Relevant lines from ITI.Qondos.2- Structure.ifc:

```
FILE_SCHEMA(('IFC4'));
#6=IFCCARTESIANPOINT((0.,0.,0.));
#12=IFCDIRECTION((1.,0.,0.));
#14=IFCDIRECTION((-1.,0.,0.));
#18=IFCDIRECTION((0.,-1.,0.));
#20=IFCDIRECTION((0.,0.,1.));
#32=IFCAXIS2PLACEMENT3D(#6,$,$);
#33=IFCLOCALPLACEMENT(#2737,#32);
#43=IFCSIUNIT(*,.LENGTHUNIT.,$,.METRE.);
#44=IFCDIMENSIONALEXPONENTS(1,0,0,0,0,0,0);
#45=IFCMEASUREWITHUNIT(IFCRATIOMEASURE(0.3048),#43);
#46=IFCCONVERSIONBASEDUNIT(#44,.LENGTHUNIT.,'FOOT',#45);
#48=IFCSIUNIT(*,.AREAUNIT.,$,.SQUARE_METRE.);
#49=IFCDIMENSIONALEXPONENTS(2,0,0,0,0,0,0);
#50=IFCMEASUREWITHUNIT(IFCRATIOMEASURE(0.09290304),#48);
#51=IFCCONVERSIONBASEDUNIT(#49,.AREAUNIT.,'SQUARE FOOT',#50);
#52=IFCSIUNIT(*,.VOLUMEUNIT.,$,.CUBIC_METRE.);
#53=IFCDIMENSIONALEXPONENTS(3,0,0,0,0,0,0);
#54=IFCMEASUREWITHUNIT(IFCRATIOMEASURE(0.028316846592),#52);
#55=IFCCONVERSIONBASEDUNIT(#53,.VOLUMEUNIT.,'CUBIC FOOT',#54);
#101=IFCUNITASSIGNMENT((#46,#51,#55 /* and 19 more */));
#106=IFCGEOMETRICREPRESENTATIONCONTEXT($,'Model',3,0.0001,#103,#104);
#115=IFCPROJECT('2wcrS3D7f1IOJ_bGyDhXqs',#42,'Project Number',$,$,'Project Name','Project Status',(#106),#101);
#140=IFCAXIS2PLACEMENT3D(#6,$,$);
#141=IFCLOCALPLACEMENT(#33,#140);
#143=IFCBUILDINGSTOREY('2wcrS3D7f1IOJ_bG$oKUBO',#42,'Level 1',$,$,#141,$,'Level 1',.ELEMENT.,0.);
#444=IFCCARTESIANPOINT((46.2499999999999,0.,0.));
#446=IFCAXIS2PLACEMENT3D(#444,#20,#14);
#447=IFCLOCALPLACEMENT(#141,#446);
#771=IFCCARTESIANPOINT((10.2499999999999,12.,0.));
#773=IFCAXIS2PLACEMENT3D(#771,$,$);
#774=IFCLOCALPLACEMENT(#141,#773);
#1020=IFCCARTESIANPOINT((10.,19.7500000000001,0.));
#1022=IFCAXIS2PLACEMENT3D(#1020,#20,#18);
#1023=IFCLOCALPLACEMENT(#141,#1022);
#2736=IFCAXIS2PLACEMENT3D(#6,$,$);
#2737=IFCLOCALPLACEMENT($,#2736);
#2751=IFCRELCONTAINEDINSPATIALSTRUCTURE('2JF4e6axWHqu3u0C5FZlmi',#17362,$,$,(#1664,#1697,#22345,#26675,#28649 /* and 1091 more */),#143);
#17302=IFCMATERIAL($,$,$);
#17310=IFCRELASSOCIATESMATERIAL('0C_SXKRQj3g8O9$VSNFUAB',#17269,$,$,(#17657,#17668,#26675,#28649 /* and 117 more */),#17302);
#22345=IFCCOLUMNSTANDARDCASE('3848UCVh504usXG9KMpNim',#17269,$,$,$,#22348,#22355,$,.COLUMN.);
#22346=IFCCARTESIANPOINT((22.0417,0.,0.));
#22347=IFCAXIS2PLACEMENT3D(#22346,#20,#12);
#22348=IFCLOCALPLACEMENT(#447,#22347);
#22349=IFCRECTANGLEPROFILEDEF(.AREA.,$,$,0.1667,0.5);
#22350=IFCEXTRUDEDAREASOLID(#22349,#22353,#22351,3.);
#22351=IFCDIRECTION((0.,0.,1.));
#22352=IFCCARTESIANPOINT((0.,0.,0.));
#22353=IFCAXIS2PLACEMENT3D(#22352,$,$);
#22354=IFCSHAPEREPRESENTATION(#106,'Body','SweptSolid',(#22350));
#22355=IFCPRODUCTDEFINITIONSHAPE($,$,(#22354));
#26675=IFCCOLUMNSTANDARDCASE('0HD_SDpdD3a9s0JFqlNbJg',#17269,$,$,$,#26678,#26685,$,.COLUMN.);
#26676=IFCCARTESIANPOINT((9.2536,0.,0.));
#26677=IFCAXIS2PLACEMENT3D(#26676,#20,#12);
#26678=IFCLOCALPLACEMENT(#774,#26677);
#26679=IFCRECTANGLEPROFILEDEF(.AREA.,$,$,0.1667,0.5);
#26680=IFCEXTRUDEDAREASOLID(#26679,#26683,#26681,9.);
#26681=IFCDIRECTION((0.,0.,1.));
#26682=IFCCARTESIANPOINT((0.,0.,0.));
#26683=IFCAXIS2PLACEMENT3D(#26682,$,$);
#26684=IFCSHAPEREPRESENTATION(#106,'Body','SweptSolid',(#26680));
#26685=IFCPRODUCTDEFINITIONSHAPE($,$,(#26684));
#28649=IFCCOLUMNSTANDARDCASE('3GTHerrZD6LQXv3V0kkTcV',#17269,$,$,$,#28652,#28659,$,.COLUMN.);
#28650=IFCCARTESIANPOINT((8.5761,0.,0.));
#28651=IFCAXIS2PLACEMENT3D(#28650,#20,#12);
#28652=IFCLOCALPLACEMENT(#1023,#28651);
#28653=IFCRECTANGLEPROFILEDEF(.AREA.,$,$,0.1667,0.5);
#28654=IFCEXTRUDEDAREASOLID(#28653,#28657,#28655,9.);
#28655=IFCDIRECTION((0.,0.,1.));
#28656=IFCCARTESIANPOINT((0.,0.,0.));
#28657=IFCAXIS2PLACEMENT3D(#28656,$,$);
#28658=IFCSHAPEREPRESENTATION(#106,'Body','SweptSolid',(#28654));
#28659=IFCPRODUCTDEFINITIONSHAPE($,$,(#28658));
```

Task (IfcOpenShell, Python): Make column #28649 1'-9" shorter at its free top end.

```python
import ifcopenshell
import ifcopenshell.util.unit

model = ifcopenshell.open("ITI.Qondos.2- Structure.ifc")
unit_scale = ifcopenshell.util.unit.calculate_unit_scale(model)

member = model.by_id(28649)
change = -21 * 0.0254 / unit_scale

# The extrusion runs towards the end named, so only its depth changes.
body = next(r for r in member.Representation.Representations if r.RepresentationIdentifier == "Body")
solid = body.Items[0]
old_length = solid.Depth
solid.Depth += change

print(f"length {old_length:g} -> {solid.Depth:g}")

model.write("ITI.Qondos.2- Structure_edited.ifc")
```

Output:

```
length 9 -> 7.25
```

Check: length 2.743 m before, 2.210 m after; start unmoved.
